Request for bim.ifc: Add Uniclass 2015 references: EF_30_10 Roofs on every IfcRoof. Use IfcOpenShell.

First a look at what the model holds.

```python
import ifcopenshell

model = ifcopenshell.open("bim.ifc")
print(model.schema)
print("classifications:", [c.Name for c in model.by_type("IfcClassification")])
for ifc_class in ("IfcDoor", "IfcRoof", "IfcStair", "IfcWall", "IfcWindow"):
    print(ifc_class, len(model.by_type(ifc_class)))
```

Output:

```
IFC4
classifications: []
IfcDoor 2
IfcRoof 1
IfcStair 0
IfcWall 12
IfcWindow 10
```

```python
import ifcopenshell
import ifcopenshell.api.classification

model = ifcopenshell.open("bim.ifc")

system = ifcopenshell.api.classification.add_classification(model, classification="Uniclass 2015")

codes = {
    "IfcRoof": ("EF_30_10", "Roofs"),
}
for ifc_class, (code, name) in codes.items():
    products = model.by_type(ifc_class)
    ifcopenshell.api.classification.add_reference(
        model, products=products, classification=system, identification=code, name=name
    )
    print(code, len(products))

model.write("bim_v2.ifc")
```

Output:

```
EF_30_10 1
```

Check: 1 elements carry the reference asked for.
